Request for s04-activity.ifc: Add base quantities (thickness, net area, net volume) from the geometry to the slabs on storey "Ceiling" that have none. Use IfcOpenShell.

First a look at what the model holds.

```python
import ifcopenshell
import ifcopenshell.util.element
import ifcopenshell.util.unit

model = ifcopenshell.open("s04-activity.ifc")
print(model.schema)
for unit_type in ("LENGTHUNIT", "AREAUNIT", "VOLUMEUNIT"):
    print(unit_type, ifcopenshell.util.unit.calculate_unit_scale(model, unit_type))
storey = next(s for s in model.by_type("IfcBuildingStorey") if s.Name == "Ceiling")
slabs = [e for e in ifcopenshell.util.element.get_decomposition(storey) if e.is_a("IfcSlab")]
for e in sorted(slabs, key=lambda e: e.id()):
    print(e.id(), e.is_a(), e.Name, list(ifcopenshell.util.element.get_psets(e, qtos_only=True)), sep=" | ")
```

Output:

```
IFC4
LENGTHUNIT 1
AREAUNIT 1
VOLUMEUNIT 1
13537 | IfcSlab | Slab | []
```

```python
import ifcopenshell
import ifcopenshell.api.pset
import ifcopenshell.geom
import ifcopenshell.util.element
import ifcopenshell.util.shape
import ifcopenshell.util.unit

model = ifcopenshell.open("s04-activity.ifc")
unit_scale = ifcopenshell.util.unit.calculate_unit_scale(model)
area_scale = ifcopenshell.util.unit.calculate_unit_scale(model, "AREAUNIT")
volume_scale = ifcopenshell.util.unit.calculate_unit_scale(model, "VOLUMEUNIT")
settings = ifcopenshell.geom.settings()

storey = next(s for s in model.by_type("IfcBuildingStorey") if s.Name == "Ceiling")
slabs = [e for e in ifcopenshell.util.element.get_decomposition(storey) if e.is_a("IfcSlab")]

for e in sorted(slabs, key=lambda e: e.id()):
    if ifcopenshell.util.element.get_psets(e, qtos_only=True, should_inherit=False):
        continue
    # Geometry comes back in metres, in the element's own axes.
    shape = ifcopenshell.geom.create_shape(settings, e)
    values = {
        "Width": ifcopenshell.util.shape.get_z(shape.geometry) / unit_scale,
        "NetArea": ifcopenshell.util.shape.get_footprint_area(shape.geometry) / area_scale,
        "NetVolume": ifcopenshell.util.shape.get_volume(shape.geometry) / volume_scale,
    }
    qto = ifcopenshell.api.pset.add_qto(model, product=e, name="Qto_SlabBaseQuantities")
    ifcopenshell.api.pset.edit_qto(model, qto=qto, properties=values)
    print(e.id(), {k: round(v, 3) for k, v in values.items()})

model.write("s04-activity_rev.ifc")
```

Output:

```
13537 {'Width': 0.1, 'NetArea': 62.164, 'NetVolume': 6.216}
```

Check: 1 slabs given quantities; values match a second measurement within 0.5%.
